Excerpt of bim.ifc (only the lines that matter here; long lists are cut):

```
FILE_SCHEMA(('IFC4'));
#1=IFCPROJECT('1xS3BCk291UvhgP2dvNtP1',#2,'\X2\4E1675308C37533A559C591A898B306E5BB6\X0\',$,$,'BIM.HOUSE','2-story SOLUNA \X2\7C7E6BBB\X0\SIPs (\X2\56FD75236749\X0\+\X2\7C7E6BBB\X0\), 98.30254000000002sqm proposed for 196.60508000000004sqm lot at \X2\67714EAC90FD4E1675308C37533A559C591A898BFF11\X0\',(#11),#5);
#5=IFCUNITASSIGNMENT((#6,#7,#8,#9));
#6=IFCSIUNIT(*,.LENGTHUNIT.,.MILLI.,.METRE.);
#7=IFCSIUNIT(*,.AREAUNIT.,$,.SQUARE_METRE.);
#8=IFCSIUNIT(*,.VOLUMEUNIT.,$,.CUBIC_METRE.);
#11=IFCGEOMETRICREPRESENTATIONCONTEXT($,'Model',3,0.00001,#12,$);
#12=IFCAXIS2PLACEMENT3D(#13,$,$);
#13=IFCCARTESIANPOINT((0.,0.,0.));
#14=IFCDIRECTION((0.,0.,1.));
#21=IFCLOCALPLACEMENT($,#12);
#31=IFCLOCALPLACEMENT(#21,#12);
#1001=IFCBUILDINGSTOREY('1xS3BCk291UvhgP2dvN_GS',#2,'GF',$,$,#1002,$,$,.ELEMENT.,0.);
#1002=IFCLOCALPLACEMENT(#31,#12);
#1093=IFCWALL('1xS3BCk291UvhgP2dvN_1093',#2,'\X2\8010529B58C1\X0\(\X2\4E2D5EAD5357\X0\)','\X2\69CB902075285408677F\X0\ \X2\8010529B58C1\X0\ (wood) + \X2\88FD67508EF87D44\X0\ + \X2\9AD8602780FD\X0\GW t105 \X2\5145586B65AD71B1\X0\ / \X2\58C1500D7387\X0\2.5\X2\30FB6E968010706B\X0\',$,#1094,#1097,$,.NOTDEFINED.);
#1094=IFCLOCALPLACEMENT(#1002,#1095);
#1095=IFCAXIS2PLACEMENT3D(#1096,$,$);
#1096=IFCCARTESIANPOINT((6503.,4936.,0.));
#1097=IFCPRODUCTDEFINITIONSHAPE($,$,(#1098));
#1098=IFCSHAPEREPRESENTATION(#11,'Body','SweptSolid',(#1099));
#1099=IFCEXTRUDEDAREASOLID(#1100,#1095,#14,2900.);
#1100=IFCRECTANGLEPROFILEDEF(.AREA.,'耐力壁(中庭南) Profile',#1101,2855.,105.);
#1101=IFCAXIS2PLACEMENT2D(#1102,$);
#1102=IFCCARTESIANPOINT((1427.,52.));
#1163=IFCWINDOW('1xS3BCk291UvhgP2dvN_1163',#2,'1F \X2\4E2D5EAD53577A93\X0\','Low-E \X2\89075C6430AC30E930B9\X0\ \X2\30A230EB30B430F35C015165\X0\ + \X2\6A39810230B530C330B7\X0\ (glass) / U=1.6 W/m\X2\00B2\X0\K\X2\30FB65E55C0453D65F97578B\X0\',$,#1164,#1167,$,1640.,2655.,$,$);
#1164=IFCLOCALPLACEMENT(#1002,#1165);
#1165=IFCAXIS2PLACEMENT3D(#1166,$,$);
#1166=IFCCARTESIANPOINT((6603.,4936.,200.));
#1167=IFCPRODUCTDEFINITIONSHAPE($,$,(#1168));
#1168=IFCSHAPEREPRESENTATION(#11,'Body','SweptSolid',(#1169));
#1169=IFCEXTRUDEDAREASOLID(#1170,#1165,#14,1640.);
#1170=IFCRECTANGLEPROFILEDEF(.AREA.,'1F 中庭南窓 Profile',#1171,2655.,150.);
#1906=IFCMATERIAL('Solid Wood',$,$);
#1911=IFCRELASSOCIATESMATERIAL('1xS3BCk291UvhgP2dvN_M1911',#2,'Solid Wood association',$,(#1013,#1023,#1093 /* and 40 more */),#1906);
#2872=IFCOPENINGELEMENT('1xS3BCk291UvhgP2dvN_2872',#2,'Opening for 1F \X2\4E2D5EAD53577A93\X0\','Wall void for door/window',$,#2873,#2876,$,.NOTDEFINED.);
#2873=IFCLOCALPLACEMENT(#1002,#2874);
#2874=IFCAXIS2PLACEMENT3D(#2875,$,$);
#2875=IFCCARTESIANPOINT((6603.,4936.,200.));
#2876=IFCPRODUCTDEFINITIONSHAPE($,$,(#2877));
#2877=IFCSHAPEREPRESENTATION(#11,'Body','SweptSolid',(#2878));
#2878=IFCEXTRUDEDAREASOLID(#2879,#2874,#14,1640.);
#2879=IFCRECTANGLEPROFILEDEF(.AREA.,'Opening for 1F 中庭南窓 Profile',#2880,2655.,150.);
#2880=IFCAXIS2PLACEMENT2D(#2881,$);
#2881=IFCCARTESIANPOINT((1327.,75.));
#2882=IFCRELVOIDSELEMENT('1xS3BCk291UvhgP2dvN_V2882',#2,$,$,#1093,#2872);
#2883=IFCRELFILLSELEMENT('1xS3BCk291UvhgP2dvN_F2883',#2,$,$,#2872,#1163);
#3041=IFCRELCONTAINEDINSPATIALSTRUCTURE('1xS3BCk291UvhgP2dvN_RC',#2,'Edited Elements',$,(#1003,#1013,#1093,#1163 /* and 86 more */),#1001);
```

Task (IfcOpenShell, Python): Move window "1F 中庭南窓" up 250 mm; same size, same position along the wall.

```python
import numpy as np
import ifcopenshell
import ifcopenshell.api.geometry
import ifcopenshell.util.placement
import ifcopenshell.util.unit

model = ifcopenshell.open("bim.ifc")
unit_scale = ifcopenshell.util.unit.calculate_unit_scale(model)

window = model.by_guid("1xS3BCk291UvhgP2dvN_1163")
opening = window.FillsVoids[0].RelatingOpeningElement
dz = 0.25 / unit_scale

shift = np.array([0.0, 0.0, dz])
# The window is not placed relative to its opening, so move both.
for product in (opening, window):
    matrix = ifcopenshell.util.placement.get_local_placement(product.ObjectPlacement)
    matrix[:3, 3] += shift
    ifcopenshell.api.geometry.edit_object_placement(model, product=product, matrix=matrix, is_si=False)

print(f"moved by {dz * unit_scale:+.3f} m")

model.write("bim_edited.ifc")
```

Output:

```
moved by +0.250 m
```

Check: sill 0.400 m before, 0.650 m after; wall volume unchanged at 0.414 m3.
